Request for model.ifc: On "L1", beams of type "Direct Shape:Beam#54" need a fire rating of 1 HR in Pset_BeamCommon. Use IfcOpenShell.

First a look at what the model holds.

```python
import ifcopenshell
import ifcopenshell.util.element

model = ifcopenshell.open("model.ifc")
print(model.schema)
storey = next(s for s in model.by_type("IfcBuildingStorey") if s.Name == "L1")
beams = [e for e in ifcopenshell.util.element.get_decomposition(storey) if e.is_a("IfcBeam")]
seen = {}
for e in beams:
    element_type = ifcopenshell.util.element.get_type(e)
    key = (element_type.Name if element_type != e and element_type else None, ifcopenshell.util.element.get_pset(e, "Pset_BeamCommon", "FireRating"))
    seen[key] = seen.get(key, 0) + 1
for (name, value), count in sorted(seen.items(), key=str):
    print(count, "x", name, "|", value)
```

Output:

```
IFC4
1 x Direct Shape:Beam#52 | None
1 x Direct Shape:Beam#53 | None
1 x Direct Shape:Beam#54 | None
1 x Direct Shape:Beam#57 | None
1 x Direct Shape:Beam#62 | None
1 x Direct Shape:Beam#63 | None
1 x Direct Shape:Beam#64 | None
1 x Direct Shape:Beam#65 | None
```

```python
import ifcopenshell
import ifcopenshell.api.pset
import ifcopenshell.util.element

model = ifcopenshell.open("model.ifc")

storey = next(s for s in model.by_type("IfcBuildingStorey") if s.Name == "L1")
beams = [e for e in ifcopenshell.util.element.get_decomposition(storey) if e.is_a("IfcBeam")]

count = 0
for e in beams:
    element_type = ifcopenshell.util.element.get_type(e)
    if element_type in (None, e) or element_type.Name != "Direct Shape:Beam#54":
        continue
    # add_pset returns the element's existing set when there is one.
    pset = ifcopenshell.api.pset.add_pset(model, product=e, name="Pset_BeamCommon")
    ifcopenshell.api.pset.edit_pset(model, pset=pset, properties={"FireRating": "1 HR"})
    count += 1

print(count, "beams updated")

model.write("model-out.ifc")
```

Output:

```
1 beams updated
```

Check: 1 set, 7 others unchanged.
